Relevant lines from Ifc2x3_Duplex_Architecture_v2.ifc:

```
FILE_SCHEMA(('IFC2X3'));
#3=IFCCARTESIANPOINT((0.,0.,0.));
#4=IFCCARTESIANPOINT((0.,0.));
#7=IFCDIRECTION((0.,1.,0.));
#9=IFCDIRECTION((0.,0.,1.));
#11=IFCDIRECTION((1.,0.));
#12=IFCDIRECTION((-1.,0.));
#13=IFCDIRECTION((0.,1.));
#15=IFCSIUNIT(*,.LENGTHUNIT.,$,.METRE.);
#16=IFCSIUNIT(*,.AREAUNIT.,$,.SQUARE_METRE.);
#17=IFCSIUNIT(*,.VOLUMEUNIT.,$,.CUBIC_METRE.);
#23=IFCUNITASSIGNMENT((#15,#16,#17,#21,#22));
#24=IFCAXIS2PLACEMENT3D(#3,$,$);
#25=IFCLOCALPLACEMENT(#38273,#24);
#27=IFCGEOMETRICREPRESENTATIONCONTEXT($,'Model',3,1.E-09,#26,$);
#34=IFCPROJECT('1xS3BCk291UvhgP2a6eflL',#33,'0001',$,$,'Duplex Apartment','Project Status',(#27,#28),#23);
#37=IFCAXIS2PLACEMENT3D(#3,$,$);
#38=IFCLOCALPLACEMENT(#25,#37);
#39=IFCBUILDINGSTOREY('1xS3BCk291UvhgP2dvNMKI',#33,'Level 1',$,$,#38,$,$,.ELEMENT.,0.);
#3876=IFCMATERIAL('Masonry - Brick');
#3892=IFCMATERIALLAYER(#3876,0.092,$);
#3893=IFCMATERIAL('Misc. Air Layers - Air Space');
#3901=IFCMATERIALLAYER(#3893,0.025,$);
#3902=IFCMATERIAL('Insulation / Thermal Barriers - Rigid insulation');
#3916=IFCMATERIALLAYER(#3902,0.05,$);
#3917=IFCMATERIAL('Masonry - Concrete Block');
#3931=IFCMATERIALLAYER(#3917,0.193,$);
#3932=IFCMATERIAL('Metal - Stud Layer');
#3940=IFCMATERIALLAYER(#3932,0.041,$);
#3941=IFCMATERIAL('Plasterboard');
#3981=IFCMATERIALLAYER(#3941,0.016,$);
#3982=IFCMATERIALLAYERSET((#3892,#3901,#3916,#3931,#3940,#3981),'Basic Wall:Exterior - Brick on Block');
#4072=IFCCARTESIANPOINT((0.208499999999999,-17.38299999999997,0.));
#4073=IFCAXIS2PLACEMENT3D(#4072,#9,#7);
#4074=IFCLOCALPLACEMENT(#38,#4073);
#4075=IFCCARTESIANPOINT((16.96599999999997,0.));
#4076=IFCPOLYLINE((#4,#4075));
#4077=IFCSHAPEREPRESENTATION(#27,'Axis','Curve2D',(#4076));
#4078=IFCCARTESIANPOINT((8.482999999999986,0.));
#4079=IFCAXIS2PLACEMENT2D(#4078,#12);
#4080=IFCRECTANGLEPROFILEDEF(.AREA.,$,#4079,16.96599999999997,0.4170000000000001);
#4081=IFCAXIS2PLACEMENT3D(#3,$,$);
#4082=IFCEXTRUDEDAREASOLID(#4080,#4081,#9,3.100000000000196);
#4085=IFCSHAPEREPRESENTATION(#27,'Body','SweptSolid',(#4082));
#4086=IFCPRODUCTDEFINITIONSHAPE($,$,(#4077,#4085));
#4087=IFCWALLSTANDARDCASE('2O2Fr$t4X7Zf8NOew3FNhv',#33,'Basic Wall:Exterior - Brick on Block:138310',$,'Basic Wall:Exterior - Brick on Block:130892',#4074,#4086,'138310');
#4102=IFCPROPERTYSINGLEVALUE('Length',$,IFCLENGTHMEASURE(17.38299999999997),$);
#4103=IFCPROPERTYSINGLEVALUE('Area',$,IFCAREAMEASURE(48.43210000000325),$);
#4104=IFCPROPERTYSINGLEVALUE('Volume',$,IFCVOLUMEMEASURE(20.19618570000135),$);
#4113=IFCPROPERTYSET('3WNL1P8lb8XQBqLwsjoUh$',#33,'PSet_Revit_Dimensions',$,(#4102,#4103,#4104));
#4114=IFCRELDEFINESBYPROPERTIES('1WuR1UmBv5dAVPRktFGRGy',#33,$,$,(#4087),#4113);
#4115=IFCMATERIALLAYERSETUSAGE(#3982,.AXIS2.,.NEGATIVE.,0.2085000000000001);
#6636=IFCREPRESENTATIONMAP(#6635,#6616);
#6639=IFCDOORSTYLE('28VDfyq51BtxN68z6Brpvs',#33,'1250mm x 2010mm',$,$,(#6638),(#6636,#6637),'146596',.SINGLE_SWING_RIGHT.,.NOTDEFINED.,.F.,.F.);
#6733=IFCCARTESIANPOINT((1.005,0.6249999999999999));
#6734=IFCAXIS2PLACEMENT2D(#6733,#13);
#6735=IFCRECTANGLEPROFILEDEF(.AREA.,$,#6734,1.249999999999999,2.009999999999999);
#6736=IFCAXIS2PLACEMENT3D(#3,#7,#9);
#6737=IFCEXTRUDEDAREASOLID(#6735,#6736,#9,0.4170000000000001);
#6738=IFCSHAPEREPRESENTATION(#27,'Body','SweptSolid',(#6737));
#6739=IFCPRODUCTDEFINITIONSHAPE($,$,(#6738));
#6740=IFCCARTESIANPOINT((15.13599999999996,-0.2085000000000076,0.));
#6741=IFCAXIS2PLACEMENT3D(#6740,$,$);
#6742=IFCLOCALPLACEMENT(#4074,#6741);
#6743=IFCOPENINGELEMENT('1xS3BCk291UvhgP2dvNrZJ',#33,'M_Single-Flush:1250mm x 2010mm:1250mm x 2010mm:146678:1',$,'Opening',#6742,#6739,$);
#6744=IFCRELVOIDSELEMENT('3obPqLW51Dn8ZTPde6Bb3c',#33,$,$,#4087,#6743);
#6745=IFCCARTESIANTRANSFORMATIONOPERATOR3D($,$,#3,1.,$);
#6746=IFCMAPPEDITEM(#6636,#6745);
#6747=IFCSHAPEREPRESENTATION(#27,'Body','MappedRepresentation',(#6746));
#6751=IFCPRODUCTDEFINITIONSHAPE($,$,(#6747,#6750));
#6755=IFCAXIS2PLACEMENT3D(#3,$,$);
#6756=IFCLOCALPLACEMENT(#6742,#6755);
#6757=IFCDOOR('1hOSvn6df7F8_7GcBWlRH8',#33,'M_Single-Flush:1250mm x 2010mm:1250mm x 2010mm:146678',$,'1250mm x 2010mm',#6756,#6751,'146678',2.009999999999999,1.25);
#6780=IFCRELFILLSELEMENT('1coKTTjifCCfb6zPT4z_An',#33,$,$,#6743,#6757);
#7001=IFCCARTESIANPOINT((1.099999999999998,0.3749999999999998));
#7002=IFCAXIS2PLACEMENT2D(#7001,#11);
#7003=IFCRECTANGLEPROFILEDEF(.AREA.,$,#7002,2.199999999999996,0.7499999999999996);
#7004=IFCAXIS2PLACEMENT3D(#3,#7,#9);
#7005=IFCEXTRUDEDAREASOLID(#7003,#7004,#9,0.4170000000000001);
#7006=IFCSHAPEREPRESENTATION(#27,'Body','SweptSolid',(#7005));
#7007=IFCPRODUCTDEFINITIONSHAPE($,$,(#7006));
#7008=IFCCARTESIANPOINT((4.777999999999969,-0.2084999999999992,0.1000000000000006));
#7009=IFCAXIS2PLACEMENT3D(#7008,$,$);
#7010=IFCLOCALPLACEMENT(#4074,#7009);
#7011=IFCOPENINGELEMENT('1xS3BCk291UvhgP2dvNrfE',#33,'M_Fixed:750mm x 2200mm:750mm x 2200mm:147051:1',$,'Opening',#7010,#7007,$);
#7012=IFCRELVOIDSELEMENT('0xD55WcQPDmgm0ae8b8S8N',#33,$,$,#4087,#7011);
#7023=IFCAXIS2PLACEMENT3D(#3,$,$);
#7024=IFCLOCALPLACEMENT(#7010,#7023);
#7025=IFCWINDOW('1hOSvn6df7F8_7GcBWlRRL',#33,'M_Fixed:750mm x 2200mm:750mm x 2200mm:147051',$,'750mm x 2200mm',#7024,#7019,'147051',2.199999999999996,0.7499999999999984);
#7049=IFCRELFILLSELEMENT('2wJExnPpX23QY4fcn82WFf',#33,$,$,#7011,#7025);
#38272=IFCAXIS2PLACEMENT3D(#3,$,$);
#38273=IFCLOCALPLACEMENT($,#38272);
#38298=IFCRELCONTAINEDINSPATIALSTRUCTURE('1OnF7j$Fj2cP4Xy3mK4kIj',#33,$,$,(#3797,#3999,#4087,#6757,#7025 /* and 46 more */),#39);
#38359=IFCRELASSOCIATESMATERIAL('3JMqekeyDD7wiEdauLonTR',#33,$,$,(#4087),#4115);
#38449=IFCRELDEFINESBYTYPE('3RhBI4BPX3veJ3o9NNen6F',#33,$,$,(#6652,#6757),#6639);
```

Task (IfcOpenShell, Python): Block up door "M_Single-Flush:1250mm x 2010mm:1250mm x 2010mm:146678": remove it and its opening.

```python
import ifcopenshell
import ifcopenshell.api.feature
import ifcopenshell.api.pset
import ifcopenshell.api.root
import ifcopenshell.geom
import ifcopenshell.util.element
import ifcopenshell.util.shape
import ifcopenshell.util.unit

model = ifcopenshell.open("Ifc2x3_Duplex_Architecture_v2.ifc")
area_scale = ifcopenshell.util.unit.calculate_unit_scale(model, "AREAUNIT")
volume_scale = ifcopenshell.util.unit.calculate_unit_scale(model, "VOLUMEUNIT")
settings = ifcopenshell.geom.settings()


def volume(element):
    """Net volume in cubic metres, openings subtracted."""
    shape = ifcopenshell.geom.create_shape(settings, element)
    return ifcopenshell.util.shape.get_volume(shape.geometry)


door = model.by_id(6757)
opening = door.FillsVoids[0].RelatingOpeningElement
wall = opening.VoidsElements[0].RelatingBuildingElement
before = volume(wall)

ifcopenshell.api.root.remove_product(model, product=door)
ifcopenshell.api.feature.remove_feature(model, feature=opening)

after = volume(wall)
thickness = 0.417  # wall thickness in metres

# Update the wall's stored quantities.
pset = model.by_id(ifcopenshell.util.element.get_pset(wall, "PSet_Revit_Dimensions", should_inherit=False)["id"])
ifcopenshell.api.pset.edit_pset(model, pset=pset, properties={
    "Area": model.create_entity("IfcAreaMeasure", after / thickness / area_scale),
    "Volume": model.create_entity("IfcVolumeMeasure", after / volume_scale),
})

print(f"wall volume {before:.3f} -> {after:.3f} m3")

model.write("Ifc2x3_Duplex_Architecture_v2_rev.ifc")
```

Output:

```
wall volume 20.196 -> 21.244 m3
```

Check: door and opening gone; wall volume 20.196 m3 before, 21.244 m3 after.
